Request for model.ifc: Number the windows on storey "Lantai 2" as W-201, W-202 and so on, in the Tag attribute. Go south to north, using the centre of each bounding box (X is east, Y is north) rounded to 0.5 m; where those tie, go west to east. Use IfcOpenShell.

First a look at what the model holds.

```python
import ifcopenshell
import ifcopenshell.util.element
import ifcopenshell.util.placement

model = ifcopenshell.open("model.ifc")
print(model.schema)
storey = next(s for s in model.by_type("IfcBuildingStorey") if s.Name == "Lantai 2")
windows = [e for e in ifcopenshell.util.element.get_decomposition(storey) if e.is_a("IfcWindow")]
for e in sorted(windows, key=lambda e: e.id()):
    origin = ifcopenshell.util.placement.get_local_placement(e.ObjectPlacement)[:3, 3]
    print(e.id(), e.Tag, e.Name, origin.round(2) + 0.0, sep=" | ")
```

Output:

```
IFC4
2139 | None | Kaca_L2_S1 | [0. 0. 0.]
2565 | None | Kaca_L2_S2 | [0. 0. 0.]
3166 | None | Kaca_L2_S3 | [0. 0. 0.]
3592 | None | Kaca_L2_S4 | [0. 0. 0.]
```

```python
import ifcopenshell
import ifcopenshell.geom
import ifcopenshell.util.element
import ifcopenshell.util.shape

model = ifcopenshell.open("model.ifc")
settings = ifcopenshell.geom.settings()
settings.set("use-world-coords", True)


def centre(element):
    shape = ifcopenshell.geom.create_shape(settings, element)
    return ifcopenshell.util.shape.get_bbox_centroid(shape.geometry)


storey = next(s for s in model.by_type("IfcBuildingStorey") if s.Name == "Lantai 2")
windows = [e for e in ifcopenshell.util.element.get_decomposition(storey) if e.is_a("IfcWindow")]

# Insertion points can sit at a corner or the storey origin, so sort by the geometry (in metres).
centres = {e: centre(e) for e in windows}
windows.sort(key=lambda e: (round(centres[e][1] / 0.5), centres[e][0]))

for i, e in enumerate(windows, start=1):
    number = f"W-2{i:02d}"
    e.Tag = number
    print(e.id(), number)

model.write("model_updated.ifc")
```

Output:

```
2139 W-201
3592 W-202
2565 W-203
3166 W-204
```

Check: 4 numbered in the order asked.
